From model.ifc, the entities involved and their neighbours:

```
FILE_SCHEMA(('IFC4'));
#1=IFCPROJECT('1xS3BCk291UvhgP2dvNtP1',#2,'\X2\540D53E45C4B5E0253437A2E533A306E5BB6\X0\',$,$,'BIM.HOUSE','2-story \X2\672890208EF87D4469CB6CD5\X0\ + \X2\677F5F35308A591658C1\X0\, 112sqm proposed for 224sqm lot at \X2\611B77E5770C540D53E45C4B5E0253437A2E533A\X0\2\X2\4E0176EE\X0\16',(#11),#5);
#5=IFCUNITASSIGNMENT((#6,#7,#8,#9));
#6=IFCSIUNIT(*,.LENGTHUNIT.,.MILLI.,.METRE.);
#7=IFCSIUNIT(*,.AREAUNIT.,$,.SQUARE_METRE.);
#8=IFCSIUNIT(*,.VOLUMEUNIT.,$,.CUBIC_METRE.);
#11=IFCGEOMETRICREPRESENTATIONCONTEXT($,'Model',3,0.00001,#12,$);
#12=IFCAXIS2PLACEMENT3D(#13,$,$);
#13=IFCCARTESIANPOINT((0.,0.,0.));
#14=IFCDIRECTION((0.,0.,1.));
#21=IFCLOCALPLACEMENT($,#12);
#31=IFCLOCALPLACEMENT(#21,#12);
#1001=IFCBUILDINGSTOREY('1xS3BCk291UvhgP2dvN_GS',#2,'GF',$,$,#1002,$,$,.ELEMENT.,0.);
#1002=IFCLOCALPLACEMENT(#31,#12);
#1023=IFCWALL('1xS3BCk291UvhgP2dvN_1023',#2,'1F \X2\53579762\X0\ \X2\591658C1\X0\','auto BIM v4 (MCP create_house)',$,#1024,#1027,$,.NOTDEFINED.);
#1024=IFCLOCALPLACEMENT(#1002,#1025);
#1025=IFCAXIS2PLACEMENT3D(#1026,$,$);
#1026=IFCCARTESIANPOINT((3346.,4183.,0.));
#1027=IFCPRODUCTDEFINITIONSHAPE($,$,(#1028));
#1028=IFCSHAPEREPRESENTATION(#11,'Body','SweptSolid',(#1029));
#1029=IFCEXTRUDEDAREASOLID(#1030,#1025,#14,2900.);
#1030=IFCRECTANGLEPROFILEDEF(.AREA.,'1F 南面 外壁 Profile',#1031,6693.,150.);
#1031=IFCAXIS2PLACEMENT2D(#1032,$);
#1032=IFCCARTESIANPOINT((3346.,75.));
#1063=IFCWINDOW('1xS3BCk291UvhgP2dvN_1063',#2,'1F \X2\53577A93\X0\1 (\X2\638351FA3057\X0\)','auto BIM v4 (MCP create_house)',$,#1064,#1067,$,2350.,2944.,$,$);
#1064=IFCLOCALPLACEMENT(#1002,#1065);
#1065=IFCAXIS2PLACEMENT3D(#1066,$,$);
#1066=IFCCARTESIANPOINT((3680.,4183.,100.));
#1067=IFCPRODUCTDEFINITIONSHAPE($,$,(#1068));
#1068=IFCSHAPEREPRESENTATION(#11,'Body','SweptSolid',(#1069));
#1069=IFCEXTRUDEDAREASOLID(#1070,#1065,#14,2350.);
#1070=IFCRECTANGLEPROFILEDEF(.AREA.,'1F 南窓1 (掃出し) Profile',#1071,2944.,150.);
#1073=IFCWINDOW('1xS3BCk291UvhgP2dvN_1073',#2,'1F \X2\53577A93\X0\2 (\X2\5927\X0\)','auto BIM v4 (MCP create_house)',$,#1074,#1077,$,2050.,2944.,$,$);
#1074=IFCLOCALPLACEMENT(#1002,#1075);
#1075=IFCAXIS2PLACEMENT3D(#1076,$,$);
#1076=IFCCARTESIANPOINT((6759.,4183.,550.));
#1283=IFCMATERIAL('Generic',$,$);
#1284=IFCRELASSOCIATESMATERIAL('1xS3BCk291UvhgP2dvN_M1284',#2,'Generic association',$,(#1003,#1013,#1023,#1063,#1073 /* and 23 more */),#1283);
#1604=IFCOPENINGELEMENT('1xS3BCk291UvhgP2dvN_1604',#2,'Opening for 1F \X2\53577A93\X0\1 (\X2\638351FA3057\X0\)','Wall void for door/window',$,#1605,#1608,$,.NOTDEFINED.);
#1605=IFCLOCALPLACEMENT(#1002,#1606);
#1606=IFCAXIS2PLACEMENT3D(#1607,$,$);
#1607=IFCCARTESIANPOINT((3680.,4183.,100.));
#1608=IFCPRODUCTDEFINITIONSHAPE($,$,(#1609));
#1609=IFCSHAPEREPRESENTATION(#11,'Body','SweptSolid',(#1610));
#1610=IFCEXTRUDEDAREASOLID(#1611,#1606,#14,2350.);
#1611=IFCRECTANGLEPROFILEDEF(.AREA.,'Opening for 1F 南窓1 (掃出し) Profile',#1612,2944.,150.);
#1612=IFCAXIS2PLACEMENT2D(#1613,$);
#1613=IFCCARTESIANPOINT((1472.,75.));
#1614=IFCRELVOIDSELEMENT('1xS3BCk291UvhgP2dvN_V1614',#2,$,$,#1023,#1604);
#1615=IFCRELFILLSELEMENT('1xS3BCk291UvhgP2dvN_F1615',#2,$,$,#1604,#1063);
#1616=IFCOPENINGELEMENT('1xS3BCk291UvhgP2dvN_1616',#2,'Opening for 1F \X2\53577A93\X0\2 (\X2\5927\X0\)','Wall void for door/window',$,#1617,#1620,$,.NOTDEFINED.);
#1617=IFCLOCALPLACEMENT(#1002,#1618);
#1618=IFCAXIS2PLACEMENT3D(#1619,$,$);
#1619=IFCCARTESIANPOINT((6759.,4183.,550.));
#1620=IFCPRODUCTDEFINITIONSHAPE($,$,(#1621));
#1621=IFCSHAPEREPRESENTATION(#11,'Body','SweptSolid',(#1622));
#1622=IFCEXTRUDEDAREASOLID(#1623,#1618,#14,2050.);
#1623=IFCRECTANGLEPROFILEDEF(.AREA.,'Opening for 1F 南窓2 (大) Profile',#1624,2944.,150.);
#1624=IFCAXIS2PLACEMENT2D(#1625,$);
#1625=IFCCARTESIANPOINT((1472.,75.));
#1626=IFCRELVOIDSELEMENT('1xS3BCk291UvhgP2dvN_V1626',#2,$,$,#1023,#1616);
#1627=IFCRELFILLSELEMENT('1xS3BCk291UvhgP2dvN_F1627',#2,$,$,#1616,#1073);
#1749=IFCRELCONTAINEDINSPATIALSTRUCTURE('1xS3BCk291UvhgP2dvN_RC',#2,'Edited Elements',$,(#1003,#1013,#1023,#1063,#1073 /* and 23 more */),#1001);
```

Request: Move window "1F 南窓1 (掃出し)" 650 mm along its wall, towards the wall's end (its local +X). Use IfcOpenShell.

```python
import ifcopenshell
import ifcopenshell.api.geometry
import ifcopenshell.util.placement
import ifcopenshell.util.unit

model = ifcopenshell.open("model.ifc")
unit_scale = ifcopenshell.util.unit.calculate_unit_scale(model)

window = model.by_guid("1xS3BCk291UvhgP2dvN_1063")
opening = window.FillsVoids[0].RelatingOpeningElement
wall = opening.VoidsElements[0].RelatingBuildingElement

wall_matrix = ifcopenshell.util.placement.get_local_placement(wall.ObjectPlacement)
shift = wall_matrix[:3, 0] * 0.65 / unit_scale
before = ifcopenshell.util.placement.get_local_placement(window.ObjectPlacement)[:3, 3].copy()

# The window is not placed relative to its opening, so move both.
for product in (opening, window):
    matrix = ifcopenshell.util.placement.get_local_placement(product.ObjectPlacement)
    matrix[:3, 3] += shift
    ifcopenshell.api.geometry.edit_object_placement(model, product=product, matrix=matrix, is_si=False)

after = ifcopenshell.util.placement.get_local_placement(window.ObjectPlacement)[:3, 3]
print("window moved by", (after - before).round(3) + 0.0)

model.write("model_updated.ifc")
```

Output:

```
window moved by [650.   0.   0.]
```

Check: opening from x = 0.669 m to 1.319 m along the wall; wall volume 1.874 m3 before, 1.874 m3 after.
